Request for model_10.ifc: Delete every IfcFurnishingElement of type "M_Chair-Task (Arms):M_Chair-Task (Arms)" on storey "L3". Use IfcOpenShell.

First a look at what the model holds.

```python
import ifcopenshell
import ifcopenshell.util.element

model = ifcopenshell.open("model_10.ifc")
print(model.schema)
storey = next(s for s in model.by_type("IfcBuildingStorey") if s.Name == "L3")
furniture = [e for e in ifcopenshell.util.element.get_decomposition(storey) if e.is_a("IfcFurnishingElement")]
seen = {}
for e in furniture:
    element_type = ifcopenshell.util.element.get_type(e)
    name = element_type.Name if element_type not in (None, e) else None
    seen[name] = seen.get(name, 0) + 1
for name, count in sorted(seen.items(), key=str):
    print(count, "x", name)
```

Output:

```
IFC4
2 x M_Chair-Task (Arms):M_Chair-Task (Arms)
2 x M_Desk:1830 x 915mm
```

```python
import ifcopenshell
import ifcopenshell.api.root
import ifcopenshell.util.element

model = ifcopenshell.open("model_10.ifc")

storey = next(s for s in model.by_type("IfcBuildingStorey") if s.Name == "L3")
furniture = [e for e in ifcopenshell.util.element.get_decomposition(storey) if e.is_a("IfcFurnishingElement")]
targets = [e for e in furniture if (t := ifcopenshell.util.element.get_type(e)) not in (None, e) and t.Name == "M_Chair-Task (Arms):M_Chair-Task (Arms)"]

for e in targets:
    ifcopenshell.api.root.remove_product(model, product=e)
print(len(targets), "removed")

model.write("model_10_v2.ifc")
```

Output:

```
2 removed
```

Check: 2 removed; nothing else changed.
